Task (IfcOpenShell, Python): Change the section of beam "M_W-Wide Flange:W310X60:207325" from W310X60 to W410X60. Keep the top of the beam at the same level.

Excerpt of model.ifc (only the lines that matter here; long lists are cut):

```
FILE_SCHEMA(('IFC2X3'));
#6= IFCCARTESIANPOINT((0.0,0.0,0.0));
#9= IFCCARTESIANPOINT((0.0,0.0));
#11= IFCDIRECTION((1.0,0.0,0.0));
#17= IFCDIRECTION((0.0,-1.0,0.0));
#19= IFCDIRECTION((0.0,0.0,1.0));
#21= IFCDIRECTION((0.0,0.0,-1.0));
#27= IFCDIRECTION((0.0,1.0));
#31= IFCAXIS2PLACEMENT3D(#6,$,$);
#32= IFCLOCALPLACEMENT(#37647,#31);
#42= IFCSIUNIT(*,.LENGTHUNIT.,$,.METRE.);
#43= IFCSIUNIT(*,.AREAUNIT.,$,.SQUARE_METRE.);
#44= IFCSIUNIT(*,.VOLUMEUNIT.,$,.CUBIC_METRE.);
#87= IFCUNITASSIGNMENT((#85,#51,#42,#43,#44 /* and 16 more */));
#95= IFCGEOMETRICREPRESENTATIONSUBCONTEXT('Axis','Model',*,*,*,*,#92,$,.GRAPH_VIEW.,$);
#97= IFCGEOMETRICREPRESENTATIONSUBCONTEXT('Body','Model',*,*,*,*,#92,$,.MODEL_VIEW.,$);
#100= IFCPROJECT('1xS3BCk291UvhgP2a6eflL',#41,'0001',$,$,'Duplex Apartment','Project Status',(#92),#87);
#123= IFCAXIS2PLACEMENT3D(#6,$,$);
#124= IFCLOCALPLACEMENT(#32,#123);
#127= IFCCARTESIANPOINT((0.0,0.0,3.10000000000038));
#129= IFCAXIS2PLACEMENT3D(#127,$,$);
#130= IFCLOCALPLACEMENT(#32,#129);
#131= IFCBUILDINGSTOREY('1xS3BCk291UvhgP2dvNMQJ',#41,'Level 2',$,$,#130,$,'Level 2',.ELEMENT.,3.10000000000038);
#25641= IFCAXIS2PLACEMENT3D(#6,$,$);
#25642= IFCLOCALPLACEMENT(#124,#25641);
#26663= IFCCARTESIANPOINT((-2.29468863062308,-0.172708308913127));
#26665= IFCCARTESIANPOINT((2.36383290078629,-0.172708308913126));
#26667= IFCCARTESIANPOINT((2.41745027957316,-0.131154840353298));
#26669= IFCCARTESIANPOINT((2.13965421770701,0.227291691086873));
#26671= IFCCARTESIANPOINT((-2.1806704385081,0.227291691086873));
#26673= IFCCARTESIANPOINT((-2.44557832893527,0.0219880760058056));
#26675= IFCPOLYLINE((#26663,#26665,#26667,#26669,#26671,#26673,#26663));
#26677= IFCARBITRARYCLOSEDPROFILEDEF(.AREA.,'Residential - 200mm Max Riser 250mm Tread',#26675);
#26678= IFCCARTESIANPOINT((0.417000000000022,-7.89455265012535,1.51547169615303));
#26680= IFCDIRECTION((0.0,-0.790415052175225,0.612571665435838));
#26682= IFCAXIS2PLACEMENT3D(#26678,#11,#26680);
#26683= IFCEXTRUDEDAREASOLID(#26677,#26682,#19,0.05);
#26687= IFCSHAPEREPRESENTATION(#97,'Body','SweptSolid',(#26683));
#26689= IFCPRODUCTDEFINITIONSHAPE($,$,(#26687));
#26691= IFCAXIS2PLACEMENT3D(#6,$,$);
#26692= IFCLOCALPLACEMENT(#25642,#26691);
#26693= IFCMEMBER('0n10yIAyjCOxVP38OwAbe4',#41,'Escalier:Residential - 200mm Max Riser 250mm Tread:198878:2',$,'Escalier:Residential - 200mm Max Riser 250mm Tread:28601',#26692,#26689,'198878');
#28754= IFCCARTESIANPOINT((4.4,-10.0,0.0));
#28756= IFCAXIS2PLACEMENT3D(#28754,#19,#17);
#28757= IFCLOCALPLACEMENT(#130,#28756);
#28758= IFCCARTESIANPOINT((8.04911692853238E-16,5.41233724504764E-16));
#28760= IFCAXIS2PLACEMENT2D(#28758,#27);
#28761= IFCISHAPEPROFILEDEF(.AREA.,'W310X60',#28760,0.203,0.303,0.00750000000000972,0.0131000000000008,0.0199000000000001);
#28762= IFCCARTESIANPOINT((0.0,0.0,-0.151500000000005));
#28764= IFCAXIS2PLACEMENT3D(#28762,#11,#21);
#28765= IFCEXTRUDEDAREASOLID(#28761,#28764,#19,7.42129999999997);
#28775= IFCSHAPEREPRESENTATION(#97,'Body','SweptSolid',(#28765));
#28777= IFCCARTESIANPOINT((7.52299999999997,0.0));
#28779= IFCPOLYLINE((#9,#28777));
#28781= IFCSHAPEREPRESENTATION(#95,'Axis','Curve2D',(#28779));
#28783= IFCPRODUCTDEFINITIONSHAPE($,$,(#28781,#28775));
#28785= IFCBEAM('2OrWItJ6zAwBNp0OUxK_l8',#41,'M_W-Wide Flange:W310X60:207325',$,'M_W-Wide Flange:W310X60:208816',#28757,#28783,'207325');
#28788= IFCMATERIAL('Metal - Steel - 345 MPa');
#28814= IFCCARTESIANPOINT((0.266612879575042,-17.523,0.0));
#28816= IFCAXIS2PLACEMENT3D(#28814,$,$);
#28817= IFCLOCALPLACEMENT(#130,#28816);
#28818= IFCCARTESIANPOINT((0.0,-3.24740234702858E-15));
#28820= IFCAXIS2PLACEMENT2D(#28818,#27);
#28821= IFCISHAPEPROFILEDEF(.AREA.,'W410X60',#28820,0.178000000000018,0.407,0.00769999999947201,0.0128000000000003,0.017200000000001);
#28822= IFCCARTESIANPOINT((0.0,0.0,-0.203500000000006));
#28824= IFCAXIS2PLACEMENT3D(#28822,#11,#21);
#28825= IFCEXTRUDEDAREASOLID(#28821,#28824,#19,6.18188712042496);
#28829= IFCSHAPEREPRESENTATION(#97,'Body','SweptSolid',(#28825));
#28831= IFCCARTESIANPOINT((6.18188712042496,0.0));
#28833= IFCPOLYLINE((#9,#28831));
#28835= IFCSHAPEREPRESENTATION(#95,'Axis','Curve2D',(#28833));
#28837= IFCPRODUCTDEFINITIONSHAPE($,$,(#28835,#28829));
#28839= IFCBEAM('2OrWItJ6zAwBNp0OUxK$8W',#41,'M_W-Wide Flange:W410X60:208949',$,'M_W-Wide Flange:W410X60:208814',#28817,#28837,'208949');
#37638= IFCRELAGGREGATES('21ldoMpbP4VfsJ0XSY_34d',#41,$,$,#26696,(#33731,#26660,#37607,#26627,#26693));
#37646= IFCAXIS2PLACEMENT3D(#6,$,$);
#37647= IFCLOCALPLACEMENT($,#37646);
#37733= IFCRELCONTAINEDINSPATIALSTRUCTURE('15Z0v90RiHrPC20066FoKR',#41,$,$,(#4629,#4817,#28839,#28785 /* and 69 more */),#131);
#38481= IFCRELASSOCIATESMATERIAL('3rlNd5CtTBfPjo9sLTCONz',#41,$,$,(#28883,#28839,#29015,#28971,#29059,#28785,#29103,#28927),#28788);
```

```python
import ifcopenshell
import ifcopenshell.util.element
import ifcopenshell.util.representation

model = ifcopenshell.open("model.ifc")

member = model.by_guid("2OrWItJ6zAwBNp0OUxK_l8")
source = next(p for p in model.by_type("IfcIShapeProfileDef") if p.ProfileName == "W410X60")

body = ifcopenshell.util.representation.get_representation(member, "Model", "Body")
solid = body.Items[0]
old_profile = solid.SweptArea

# Copy the section's sizes but keep this member's own profile position.
profile = ifcopenshell.util.element.copy(model, source)
# Profiles are centred, so shift by half the change in depth to hold the top.
shift = (old_profile.OverallDepth - profile.OverallDepth) / 2
x, y = old_profile.Position.Location.Coordinates
up = (-1.0, 0.0)  # upwards, in the solid's own plane
location = model.createIfcCartesianPoint((x + up[0] * shift, y + up[1] * shift))
profile.Position = model.createIfcAxis2Placement2D(location, old_profile.Position.RefDirection)
solid.SweptArea = profile
if not model.get_total_inverses(old_profile):
    ifcopenshell.util.element.remove_deep2(model, old_profile)
member.Name = member.Name.replace("W310X60", "W410X60")
member.ObjectType = member.ObjectType.replace("W310X60", "W410X60")

print(solid.SweptArea)

model.write("model_edited.ifc")
```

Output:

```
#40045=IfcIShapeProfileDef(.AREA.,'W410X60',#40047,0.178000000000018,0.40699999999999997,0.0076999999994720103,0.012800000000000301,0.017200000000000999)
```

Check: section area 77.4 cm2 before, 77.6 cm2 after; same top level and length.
